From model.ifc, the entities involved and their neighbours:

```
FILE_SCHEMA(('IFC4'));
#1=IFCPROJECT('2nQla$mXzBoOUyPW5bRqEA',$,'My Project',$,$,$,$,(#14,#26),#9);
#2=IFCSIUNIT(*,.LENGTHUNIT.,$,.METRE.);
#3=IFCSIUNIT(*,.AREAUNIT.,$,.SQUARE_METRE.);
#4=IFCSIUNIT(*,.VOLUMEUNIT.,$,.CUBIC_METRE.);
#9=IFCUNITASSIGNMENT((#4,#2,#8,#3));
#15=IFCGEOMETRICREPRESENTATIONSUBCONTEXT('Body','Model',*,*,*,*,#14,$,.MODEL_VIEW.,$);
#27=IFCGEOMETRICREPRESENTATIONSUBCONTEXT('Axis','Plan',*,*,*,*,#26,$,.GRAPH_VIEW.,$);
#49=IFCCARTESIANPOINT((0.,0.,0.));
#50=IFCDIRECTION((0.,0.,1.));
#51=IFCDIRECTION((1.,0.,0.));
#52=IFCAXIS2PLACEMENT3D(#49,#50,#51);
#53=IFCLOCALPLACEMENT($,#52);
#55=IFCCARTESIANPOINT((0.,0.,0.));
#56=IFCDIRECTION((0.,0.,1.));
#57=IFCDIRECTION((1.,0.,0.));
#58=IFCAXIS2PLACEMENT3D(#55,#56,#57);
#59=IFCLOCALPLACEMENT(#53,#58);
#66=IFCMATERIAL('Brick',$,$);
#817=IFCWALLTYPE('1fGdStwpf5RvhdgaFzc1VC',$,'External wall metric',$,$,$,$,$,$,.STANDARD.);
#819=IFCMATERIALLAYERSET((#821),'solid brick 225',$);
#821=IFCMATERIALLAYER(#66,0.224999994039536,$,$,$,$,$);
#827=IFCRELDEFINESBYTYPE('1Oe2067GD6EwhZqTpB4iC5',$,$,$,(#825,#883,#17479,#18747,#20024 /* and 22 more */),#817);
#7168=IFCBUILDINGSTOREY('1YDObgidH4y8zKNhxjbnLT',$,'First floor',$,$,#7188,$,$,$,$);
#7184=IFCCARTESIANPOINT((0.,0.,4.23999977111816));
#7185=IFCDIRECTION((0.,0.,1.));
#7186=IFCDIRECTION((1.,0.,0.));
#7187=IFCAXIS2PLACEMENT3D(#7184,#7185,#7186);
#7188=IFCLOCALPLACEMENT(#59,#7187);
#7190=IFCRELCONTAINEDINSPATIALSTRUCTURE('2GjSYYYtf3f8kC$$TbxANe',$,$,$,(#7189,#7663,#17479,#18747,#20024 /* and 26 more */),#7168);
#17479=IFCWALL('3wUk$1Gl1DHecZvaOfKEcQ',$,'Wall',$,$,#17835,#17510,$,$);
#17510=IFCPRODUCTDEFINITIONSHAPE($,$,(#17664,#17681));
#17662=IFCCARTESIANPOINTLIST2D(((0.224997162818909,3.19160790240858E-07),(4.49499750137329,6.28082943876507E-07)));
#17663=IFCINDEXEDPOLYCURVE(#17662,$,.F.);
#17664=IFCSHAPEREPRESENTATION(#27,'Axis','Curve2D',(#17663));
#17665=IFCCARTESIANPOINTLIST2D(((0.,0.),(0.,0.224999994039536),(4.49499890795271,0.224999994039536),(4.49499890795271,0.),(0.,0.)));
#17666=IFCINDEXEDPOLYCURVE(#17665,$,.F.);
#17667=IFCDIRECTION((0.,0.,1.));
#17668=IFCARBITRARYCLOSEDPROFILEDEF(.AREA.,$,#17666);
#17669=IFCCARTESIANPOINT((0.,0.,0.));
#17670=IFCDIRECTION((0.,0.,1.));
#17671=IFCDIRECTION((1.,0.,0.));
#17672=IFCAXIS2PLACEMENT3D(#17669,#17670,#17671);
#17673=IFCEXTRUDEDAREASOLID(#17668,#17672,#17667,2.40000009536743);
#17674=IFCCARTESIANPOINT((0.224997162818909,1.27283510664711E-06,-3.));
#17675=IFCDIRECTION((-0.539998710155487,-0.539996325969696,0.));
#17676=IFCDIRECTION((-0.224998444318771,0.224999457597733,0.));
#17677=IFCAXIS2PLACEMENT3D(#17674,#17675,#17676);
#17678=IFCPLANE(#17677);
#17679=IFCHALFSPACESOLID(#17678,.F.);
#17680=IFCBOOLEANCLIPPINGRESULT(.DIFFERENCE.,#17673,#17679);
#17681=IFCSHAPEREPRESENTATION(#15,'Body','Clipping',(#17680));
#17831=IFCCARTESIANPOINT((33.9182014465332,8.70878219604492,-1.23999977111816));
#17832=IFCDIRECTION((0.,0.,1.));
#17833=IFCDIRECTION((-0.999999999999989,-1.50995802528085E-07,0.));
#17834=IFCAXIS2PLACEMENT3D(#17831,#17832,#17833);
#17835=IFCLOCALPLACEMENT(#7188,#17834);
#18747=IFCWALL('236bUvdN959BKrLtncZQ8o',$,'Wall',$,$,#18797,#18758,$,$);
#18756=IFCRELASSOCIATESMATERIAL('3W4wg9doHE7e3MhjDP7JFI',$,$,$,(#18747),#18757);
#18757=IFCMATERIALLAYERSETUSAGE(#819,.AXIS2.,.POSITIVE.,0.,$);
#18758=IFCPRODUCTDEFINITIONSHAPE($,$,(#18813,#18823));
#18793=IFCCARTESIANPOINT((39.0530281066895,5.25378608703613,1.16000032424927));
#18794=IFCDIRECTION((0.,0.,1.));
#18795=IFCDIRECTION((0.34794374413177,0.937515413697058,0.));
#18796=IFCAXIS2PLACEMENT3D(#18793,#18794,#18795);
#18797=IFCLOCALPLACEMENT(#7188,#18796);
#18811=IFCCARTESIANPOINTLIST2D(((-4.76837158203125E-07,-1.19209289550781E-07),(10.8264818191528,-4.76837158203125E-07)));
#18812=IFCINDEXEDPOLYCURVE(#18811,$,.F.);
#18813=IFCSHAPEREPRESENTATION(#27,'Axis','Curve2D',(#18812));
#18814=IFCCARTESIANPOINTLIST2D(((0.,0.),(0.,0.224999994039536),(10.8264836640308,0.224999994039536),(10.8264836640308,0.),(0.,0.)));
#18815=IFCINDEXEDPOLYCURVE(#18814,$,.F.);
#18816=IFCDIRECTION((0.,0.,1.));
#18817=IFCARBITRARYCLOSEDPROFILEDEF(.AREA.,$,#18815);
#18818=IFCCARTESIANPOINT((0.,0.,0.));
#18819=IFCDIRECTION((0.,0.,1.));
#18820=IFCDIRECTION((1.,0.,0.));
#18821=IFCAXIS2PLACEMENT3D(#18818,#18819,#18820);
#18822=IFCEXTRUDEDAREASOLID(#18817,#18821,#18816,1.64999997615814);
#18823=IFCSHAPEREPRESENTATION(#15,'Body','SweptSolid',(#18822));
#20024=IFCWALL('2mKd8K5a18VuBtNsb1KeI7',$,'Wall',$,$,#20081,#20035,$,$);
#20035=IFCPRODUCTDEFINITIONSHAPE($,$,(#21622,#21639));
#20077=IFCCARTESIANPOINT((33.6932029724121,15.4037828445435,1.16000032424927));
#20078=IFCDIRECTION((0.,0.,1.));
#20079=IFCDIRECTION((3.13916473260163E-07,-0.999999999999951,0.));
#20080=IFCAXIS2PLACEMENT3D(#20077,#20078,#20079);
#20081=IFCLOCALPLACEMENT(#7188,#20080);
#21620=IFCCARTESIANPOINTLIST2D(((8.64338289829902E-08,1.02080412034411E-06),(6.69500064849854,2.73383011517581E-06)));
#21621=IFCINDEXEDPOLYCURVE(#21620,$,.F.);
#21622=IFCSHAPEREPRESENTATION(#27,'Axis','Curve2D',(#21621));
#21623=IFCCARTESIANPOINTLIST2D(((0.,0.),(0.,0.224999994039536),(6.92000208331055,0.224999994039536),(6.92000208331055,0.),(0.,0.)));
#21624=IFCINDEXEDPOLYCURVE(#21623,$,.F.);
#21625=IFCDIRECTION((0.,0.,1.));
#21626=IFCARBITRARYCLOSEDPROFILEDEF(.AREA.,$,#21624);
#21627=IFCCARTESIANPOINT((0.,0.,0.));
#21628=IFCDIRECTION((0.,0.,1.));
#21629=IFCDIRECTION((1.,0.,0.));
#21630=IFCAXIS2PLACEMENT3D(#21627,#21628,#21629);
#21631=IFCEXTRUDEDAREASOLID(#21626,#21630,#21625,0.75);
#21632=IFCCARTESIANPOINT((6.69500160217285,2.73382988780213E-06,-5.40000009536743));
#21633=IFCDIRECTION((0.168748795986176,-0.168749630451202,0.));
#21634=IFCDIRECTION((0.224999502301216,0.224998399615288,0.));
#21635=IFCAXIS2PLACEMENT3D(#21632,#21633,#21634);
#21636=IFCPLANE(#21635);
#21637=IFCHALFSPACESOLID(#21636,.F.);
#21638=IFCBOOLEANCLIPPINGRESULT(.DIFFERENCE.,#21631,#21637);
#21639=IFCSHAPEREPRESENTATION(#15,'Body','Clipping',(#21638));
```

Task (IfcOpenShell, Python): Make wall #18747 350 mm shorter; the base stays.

```python
import ifcopenshell
import ifcopenshell.geom
import ifcopenshell.util.representation
import ifcopenshell.util.shape

model = ifcopenshell.open("model.ifc")
settings = ifcopenshell.geom.settings()


def volume(element):
    """Net volume in cubic metres, openings subtracted."""
    shape = ifcopenshell.geom.create_shape(settings, element)
    return ifcopenshell.util.shape.get_volume(shape.geometry)


wall = model.by_id(18747)
before = volume(wall)

body = ifcopenshell.util.representation.get_representation(wall, "Model", "Body")
solid = body.Items[0]
old_height = solid.Depth
solid.Depth -= 0.35
after = volume(wall)

print(f"height {old_height:g} -> {solid.Depth:g}, volume {before:.3f} -> {after:.3f} m3")

model.write("model-out.ifc")
```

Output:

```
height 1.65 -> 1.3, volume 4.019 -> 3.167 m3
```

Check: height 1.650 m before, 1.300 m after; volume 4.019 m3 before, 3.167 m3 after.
